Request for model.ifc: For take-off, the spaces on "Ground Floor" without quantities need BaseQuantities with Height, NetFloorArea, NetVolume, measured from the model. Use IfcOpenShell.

First a look at what the model holds.

```python
import ifcopenshell
import ifcopenshell.util.element
import ifcopenshell.util.unit

model = ifcopenshell.open("model.ifc")
print(model.schema)
for unit_type in ("LENGTHUNIT", "AREAUNIT", "VOLUMEUNIT"):
    print(unit_type, ifcopenshell.util.unit.calculate_unit_scale(model, unit_type))
storey = next(s for s in model.by_type("IfcBuildingStorey") if s.Name == "Ground Floor")
spaces = [e for e in ifcopenshell.util.element.get_decomposition(storey) if e.is_a("IfcSpace")]
for e in sorted(spaces, key=lambda e: e.id()):
    print(e.id(), e.is_a(), e.Name, list(ifcopenshell.util.element.get_psets(e, qtos_only=True)), sep=" | ")
```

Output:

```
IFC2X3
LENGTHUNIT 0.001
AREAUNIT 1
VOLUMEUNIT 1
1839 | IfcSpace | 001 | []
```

```python
import ifcopenshell
import ifcopenshell.api.pset
import ifcopenshell.geom
import ifcopenshell.util.element
import ifcopenshell.util.shape
import ifcopenshell.util.unit

model = ifcopenshell.open("model.ifc")
unit_scale = ifcopenshell.util.unit.calculate_unit_scale(model)
area_scale = ifcopenshell.util.unit.calculate_unit_scale(model, "AREAUNIT")
volume_scale = ifcopenshell.util.unit.calculate_unit_scale(model, "VOLUMEUNIT")
settings = ifcopenshell.geom.settings()

storey = next(s for s in model.by_type("IfcBuildingStorey") if s.Name == "Ground Floor")
spaces = [e for e in ifcopenshell.util.element.get_decomposition(storey) if e.is_a("IfcSpace")]

for e in sorted(spaces, key=lambda e: e.id()):
    if ifcopenshell.util.element.get_psets(e, qtos_only=True, should_inherit=False):
        continue
    # Geometry comes back in metres, in the element's own axes.
    shape = ifcopenshell.geom.create_shape(settings, e)
    values = {
        "Height": ifcopenshell.util.shape.get_z(shape.geometry) / unit_scale,
        "NetFloorArea": ifcopenshell.util.shape.get_footprint_area(shape.geometry) / area_scale,
        "NetVolume": ifcopenshell.util.shape.get_volume(shape.geometry) / volume_scale,
    }
    qto = ifcopenshell.api.pset.add_qto(model, product=e, name="BaseQuantities")
    ifcopenshell.api.pset.edit_qto(model, qto=qto, properties=values)
    print(e.id(), {k: round(v, 3) for k, v in values.items()})

model.write("model_updated.ifc")
```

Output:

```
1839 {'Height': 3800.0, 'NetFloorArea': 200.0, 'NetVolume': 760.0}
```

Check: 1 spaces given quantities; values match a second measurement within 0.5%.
